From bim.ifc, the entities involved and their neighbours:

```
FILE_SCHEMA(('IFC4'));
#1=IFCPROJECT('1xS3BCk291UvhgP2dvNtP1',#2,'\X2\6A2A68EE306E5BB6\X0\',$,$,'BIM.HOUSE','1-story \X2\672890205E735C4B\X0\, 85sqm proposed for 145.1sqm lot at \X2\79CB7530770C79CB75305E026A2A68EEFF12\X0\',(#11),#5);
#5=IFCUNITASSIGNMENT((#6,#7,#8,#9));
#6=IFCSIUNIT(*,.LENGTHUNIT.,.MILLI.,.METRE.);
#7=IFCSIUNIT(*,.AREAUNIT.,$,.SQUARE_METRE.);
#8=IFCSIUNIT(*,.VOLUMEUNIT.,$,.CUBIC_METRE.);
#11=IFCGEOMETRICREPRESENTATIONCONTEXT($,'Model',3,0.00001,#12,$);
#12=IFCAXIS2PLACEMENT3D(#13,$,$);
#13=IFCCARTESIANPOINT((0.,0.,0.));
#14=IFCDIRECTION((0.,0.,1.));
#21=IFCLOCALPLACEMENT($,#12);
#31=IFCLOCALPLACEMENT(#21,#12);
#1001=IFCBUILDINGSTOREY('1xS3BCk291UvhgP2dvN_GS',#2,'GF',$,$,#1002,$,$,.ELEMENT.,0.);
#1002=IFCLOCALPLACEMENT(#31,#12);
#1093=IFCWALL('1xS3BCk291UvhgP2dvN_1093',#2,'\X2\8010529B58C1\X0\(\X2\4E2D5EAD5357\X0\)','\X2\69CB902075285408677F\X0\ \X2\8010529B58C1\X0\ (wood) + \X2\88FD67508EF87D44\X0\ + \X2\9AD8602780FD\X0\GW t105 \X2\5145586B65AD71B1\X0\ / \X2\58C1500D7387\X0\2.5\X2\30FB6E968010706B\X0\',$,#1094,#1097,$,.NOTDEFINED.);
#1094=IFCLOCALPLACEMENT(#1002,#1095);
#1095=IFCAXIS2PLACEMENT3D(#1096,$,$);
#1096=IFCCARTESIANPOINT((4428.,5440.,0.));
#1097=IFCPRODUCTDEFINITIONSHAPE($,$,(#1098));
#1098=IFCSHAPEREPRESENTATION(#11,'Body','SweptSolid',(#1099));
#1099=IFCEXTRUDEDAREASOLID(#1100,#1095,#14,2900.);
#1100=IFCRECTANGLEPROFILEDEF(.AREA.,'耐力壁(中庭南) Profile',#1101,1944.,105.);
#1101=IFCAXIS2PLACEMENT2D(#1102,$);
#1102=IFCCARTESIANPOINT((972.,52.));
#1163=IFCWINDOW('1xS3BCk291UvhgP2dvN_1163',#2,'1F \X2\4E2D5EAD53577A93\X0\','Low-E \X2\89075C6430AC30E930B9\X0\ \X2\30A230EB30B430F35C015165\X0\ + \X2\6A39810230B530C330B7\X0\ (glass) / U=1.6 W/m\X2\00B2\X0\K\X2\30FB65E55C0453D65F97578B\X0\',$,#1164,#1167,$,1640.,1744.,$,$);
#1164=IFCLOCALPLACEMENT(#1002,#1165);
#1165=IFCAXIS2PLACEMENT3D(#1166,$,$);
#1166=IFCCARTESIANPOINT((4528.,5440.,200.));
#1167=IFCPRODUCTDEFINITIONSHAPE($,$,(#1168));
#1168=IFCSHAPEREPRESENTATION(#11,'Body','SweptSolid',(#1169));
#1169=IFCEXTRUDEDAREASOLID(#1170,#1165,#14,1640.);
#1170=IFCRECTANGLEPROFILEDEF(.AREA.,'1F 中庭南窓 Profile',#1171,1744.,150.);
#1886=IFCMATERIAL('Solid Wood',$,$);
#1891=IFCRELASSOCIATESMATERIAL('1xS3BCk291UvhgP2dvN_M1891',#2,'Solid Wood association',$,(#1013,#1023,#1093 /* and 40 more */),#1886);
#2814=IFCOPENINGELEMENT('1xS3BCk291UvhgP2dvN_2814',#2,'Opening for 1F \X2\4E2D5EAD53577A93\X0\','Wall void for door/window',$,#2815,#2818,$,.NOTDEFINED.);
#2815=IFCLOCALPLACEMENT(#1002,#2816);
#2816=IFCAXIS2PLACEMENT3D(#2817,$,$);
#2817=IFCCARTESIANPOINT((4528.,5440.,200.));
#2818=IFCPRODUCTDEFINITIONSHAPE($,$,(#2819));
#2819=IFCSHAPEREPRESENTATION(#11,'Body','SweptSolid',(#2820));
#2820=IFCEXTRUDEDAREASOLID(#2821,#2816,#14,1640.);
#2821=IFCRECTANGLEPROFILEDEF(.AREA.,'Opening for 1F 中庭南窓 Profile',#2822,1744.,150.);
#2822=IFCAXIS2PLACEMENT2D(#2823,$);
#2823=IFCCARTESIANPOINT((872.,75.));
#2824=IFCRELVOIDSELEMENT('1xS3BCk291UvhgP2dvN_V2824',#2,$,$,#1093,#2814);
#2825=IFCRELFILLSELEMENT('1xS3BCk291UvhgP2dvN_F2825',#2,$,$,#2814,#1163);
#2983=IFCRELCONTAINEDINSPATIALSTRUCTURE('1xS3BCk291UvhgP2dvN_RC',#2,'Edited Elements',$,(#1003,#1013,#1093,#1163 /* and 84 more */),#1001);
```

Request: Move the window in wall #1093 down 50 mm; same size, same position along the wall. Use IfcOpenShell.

```python
import numpy as np
import ifcopenshell
import ifcopenshell.api.geometry
import ifcopenshell.util.placement
import ifcopenshell.util.unit

model = ifcopenshell.open("bim.ifc")
unit_scale = ifcopenshell.util.unit.calculate_unit_scale(model)

window = model.by_guid("1xS3BCk291UvhgP2dvN_1163")
opening = window.FillsVoids[0].RelatingOpeningElement
dz = -0.05 / unit_scale

shift = np.array([0.0, 0.0, dz])
# The window is not placed relative to its opening, so move both.
for product in (opening, window):
    matrix = ifcopenshell.util.placement.get_local_placement(product.ObjectPlacement)
    matrix[:3, 3] += shift
    ifcopenshell.api.geometry.edit_object_placement(model, product=product, matrix=matrix, is_si=False)

print(f"moved by {dz * unit_scale:+.3f} m")

model.write("bim-out.ifc")
```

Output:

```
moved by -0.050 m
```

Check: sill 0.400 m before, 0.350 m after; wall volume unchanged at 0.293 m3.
